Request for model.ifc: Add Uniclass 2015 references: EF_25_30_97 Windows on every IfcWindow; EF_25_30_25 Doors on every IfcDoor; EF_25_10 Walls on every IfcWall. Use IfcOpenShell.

First a look at what the model holds.

```python
import ifcopenshell

model = ifcopenshell.open("model.ifc")
print(model.schema)
print("classifications:", [c.Name for c in model.by_type("IfcClassification")])
for ifc_class in ("IfcDoor", "IfcRoof", "IfcStair", "IfcWall", "IfcWindow"):
    print(ifc_class, len(model.by_type(ifc_class)))
```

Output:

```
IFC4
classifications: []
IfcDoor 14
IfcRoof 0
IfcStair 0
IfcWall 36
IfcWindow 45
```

```python
import ifcopenshell
import ifcopenshell.api.classification

model = ifcopenshell.open("model.ifc")

system = ifcopenshell.api.classification.add_classification(model, classification="Uniclass 2015")

codes = {
    "IfcWindow": ("EF_25_30_97", "Windows"),
    "IfcDoor": ("EF_25_30_25", "Doors"),
    "IfcWall": ("EF_25_10", "Walls"),
}
for ifc_class, (code, name) in codes.items():
    products = model.by_type(ifc_class)
    ifcopenshell.api.classification.add_reference(
        model, products=products, classification=system, identification=code, name=name
    )
    print(code, len(products))

model.write("model_edited.ifc")
```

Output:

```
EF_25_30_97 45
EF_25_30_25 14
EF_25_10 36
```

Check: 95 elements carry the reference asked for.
